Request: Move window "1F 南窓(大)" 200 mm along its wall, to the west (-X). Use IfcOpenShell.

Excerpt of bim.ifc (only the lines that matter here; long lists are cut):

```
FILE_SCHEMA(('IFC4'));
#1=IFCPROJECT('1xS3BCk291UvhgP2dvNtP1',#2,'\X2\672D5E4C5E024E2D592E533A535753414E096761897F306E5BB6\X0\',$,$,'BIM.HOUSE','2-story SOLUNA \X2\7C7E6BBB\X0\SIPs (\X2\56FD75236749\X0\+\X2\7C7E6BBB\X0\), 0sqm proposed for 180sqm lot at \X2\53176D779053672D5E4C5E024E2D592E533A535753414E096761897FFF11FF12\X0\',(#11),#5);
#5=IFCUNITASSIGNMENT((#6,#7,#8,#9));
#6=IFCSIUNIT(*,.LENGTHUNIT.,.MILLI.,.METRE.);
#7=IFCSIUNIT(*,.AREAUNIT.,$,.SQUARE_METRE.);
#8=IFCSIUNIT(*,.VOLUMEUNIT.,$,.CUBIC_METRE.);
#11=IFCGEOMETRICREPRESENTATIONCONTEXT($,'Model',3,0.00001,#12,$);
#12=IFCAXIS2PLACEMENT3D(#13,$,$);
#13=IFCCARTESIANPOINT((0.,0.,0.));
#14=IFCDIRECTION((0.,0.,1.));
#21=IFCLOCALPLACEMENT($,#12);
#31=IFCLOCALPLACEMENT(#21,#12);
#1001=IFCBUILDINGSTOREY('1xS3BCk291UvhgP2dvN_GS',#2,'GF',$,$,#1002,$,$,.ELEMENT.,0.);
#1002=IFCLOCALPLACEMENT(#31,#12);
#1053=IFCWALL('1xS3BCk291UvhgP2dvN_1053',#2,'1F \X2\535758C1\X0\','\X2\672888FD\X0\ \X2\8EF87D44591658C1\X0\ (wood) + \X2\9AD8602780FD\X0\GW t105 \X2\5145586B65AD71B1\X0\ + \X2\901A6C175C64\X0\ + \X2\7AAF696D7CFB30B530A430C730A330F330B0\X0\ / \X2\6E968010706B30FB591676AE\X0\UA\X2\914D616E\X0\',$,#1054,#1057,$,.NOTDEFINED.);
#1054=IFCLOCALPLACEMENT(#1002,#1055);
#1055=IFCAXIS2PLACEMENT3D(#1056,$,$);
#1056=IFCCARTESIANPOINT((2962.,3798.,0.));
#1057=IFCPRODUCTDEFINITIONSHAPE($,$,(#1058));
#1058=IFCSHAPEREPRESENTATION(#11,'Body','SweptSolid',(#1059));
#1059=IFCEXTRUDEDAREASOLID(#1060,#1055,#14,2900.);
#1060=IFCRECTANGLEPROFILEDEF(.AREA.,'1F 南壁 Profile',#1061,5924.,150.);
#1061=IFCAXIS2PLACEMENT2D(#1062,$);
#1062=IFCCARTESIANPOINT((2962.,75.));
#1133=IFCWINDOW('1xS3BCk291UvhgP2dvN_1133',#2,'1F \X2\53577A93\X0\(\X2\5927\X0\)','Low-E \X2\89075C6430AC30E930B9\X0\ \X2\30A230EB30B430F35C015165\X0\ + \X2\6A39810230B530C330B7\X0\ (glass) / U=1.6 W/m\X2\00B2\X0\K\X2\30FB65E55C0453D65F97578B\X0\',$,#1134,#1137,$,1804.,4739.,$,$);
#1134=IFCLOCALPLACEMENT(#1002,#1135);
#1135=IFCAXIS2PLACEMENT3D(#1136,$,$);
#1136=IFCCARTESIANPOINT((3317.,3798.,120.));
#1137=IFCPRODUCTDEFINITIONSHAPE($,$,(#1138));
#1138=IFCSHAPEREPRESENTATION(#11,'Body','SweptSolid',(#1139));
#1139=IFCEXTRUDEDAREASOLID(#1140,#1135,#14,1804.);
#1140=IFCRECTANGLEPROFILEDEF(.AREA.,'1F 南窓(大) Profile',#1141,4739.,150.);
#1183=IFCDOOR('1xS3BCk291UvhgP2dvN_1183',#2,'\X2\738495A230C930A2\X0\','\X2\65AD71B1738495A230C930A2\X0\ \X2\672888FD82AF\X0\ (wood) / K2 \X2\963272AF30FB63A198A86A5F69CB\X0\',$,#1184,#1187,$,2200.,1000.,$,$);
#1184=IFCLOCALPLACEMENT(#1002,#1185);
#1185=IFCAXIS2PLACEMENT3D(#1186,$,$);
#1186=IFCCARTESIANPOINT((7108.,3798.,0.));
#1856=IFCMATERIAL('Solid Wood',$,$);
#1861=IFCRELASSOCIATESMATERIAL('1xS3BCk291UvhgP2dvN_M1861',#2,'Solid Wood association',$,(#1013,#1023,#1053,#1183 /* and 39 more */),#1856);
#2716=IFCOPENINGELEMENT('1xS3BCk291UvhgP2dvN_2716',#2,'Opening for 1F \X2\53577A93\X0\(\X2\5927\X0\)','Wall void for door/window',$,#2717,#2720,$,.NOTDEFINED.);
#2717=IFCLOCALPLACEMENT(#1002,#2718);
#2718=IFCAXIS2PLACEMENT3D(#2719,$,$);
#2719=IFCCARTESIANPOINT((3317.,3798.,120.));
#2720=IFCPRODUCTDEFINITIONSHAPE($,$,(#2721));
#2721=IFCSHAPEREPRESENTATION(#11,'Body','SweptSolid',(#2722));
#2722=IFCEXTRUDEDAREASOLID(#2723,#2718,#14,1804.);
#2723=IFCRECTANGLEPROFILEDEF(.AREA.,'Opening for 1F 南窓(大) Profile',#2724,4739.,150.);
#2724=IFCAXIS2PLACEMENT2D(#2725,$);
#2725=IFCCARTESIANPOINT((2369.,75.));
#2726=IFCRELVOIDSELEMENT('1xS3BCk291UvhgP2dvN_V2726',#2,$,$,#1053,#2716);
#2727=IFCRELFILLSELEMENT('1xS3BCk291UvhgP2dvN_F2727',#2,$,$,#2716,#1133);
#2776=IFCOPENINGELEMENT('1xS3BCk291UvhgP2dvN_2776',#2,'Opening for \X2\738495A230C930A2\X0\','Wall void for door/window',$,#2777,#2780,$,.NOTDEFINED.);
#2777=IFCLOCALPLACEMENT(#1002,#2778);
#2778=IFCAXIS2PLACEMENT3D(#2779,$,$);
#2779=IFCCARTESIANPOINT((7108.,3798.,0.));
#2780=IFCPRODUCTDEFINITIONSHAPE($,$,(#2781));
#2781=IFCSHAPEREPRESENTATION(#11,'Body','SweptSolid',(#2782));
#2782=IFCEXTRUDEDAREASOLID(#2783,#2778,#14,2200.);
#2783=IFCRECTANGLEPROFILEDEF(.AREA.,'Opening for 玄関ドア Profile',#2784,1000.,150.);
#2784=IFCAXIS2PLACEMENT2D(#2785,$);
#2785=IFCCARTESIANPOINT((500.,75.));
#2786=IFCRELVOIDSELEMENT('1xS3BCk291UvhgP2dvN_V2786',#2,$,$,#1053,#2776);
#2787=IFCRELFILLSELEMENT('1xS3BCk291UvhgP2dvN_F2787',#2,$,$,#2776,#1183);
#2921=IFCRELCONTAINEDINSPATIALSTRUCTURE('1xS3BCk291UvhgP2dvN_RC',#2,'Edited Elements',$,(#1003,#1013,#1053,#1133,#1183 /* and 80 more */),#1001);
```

```python
import ifcopenshell
import ifcopenshell.api.geometry
import ifcopenshell.util.placement
import ifcopenshell.util.unit

model = ifcopenshell.open("bim.ifc")
unit_scale = ifcopenshell.util.unit.calculate_unit_scale(model)

window = model.by_id(1133)
opening = window.FillsVoids[0].RelatingOpeningElement
wall = opening.VoidsElements[0].RelatingBuildingElement

wall_matrix = ifcopenshell.util.placement.get_local_placement(wall.ObjectPlacement)
shift = wall_matrix[:3, 0] * -0.2 / unit_scale
before = ifcopenshell.util.placement.get_local_placement(window.ObjectPlacement)[:3, 3].copy()

# The window is not placed relative to its opening, so move both.
for product in (opening, window):
    matrix = ifcopenshell.util.placement.get_local_placement(product.ObjectPlacement)
    matrix[:3, 3] += shift
    ifcopenshell.api.geometry.edit_object_placement(model, product=product, matrix=matrix, is_si=False)

after = ifcopenshell.util.placement.get_local_placement(window.ObjectPlacement)[:3, 3]
print("window moved by", (after - before).round(3) + 0.0)

model.write("bim_rev.ifc")
```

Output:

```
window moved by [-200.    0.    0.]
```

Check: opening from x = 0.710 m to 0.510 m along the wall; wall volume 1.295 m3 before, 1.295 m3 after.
